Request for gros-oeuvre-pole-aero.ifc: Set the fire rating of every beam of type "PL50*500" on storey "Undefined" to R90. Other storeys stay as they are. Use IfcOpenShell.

First a look at what the model holds.

```python
import ifcopenshell
import ifcopenshell.util.element

model = ifcopenshell.open("gros-oeuvre-pole-aero.ifc")
print(model.schema)
storey = next(s for s in model.by_type("IfcBuildingStorey") if s.Name == "Undefined")
beams = [e for e in ifcopenshell.util.element.get_decomposition(storey) if e.is_a("IfcBeam")]
seen = {}
for e in beams:
    element_type = ifcopenshell.util.element.get_type(e)
    key = (element_type.Name if element_type != e and element_type else None, ifcopenshell.util.element.get_pset(e, "Pset_BeamCommon", "FireRating"))
    seen[key] = seen.get(key, 0) + 1
for (name, value), count in sorted(seen.items(), key=str):
    print(count, "x", name, "|", value)
```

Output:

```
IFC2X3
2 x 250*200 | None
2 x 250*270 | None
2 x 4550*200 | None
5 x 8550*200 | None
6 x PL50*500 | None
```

```python
import ifcopenshell
import ifcopenshell.api.pset
import ifcopenshell.util.element

model = ifcopenshell.open("gros-oeuvre-pole-aero.ifc")

storey = next(s for s in model.by_type("IfcBuildingStorey") if s.Name == "Undefined")
beams = [e for e in ifcopenshell.util.element.get_decomposition(storey) if e.is_a("IfcBeam")]

count = 0
for e in beams:
    element_type = ifcopenshell.util.element.get_type(e)
    if element_type in (None, e) or element_type.Name != "PL50*500":
        continue
    found = ifcopenshell.util.element.get_pset(e, "Pset_BeamCommon", should_inherit=False)
    if found:
        pset = model.by_id(found["id"])
        if len(ifcopenshell.util.element.get_elements_by_pset(pset)) > 1:
            pset = ifcopenshell.api.pset.unshare_pset(model, products=[e], pset=pset)[0]
    else:
        pset = ifcopenshell.api.pset.add_pset(model, product=e, name="Pset_BeamCommon")
    ifcopenshell.api.pset.edit_pset(model, pset=pset, properties={"FireRating": "R90"})
    count += 1

print(count, "beams updated")

model.write("gros-oeuvre-pole-aero_rev.ifc")
```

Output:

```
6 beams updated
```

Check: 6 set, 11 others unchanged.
